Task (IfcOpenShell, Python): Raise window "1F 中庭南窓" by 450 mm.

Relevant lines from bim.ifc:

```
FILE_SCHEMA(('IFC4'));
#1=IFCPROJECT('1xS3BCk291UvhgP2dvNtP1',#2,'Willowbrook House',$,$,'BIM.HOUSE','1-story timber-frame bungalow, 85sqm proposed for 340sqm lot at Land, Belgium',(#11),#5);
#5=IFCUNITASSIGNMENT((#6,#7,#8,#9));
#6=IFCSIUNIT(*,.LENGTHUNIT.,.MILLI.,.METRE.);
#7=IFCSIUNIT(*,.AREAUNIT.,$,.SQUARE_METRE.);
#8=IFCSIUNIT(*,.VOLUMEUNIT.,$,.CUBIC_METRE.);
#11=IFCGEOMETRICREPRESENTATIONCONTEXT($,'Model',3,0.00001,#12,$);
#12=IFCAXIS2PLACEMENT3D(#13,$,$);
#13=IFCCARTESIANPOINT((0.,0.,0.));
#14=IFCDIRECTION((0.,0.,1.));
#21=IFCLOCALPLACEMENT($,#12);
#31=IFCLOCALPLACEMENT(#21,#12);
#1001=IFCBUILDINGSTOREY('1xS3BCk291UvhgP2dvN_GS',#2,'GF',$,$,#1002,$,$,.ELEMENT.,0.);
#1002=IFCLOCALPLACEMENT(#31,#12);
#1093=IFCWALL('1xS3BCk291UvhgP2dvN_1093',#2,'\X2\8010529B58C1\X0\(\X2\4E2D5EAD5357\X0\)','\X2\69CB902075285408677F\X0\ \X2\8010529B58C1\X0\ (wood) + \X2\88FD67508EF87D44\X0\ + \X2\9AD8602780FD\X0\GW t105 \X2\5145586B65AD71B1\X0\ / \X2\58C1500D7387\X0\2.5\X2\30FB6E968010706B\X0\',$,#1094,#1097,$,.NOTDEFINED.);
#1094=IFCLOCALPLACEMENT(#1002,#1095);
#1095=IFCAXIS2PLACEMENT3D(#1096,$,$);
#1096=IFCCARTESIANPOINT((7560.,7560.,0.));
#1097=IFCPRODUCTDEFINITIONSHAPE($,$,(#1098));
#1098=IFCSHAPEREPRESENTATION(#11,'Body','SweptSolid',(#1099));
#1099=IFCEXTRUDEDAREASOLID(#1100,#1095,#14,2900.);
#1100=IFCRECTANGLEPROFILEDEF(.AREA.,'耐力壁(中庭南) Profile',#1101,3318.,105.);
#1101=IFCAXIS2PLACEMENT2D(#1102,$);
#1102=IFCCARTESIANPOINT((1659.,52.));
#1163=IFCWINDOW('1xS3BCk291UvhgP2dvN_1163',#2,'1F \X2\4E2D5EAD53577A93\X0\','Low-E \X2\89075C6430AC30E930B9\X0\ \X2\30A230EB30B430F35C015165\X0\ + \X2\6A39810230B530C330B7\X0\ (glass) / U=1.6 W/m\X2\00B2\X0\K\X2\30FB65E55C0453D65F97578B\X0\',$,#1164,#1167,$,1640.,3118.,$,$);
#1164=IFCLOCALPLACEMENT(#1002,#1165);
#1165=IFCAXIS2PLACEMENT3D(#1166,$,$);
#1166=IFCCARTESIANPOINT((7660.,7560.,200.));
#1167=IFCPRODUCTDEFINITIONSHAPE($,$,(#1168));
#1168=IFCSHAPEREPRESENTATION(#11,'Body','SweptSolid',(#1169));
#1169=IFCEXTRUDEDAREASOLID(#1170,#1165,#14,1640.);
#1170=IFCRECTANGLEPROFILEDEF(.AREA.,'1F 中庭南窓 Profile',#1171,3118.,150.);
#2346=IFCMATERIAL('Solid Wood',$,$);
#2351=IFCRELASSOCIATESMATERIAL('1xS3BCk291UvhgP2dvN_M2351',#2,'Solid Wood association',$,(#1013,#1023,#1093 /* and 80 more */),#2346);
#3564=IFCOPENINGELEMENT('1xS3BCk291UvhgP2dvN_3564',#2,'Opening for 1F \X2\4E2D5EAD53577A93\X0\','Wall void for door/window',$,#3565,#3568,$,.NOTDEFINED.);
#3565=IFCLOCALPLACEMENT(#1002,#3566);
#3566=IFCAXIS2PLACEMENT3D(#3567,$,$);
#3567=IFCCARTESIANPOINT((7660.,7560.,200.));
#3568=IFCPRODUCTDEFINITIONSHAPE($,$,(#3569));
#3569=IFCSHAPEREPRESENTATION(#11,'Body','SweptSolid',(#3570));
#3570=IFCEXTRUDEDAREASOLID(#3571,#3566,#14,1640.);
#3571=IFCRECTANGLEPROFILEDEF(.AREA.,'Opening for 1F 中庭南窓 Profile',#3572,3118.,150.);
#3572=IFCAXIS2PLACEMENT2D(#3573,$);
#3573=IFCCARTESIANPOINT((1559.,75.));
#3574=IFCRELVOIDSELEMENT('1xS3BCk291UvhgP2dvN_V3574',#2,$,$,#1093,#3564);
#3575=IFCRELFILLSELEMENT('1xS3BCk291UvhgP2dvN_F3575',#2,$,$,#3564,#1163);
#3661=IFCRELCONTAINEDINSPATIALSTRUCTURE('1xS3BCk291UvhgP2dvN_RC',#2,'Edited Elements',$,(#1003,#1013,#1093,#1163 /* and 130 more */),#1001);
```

```python
import numpy as np
import ifcopenshell
import ifcopenshell.api.geometry
import ifcopenshell.util.placement
import ifcopenshell.util.unit

model = ifcopenshell.open("bim.ifc")
unit_scale = ifcopenshell.util.unit.calculate_unit_scale(model)

window = model.by_guid("1xS3BCk291UvhgP2dvN_1163")
opening = window.FillsVoids[0].RelatingOpeningElement
dz = 450.0

shift = np.array([0.0, 0.0, dz])
# The window is not placed relative to its opening, so move both.
for product in (opening, window):
    matrix = ifcopenshell.util.placement.get_local_placement(product.ObjectPlacement)
    matrix[:3, 3] += shift
    ifcopenshell.api.geometry.edit_object_placement(model, product=product, matrix=matrix, is_si=False)

print(f"moved by {dz * unit_scale:+.3f} m")

model.write("bim_rev.ifc")
```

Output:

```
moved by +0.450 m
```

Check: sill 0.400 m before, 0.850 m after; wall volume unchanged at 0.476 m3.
